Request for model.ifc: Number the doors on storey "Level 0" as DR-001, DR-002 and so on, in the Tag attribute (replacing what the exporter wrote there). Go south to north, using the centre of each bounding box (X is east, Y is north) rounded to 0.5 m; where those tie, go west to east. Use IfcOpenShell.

First a look at what the model holds.

```python
import ifcopenshell
import ifcopenshell.util.element
import ifcopenshell.util.placement

model = ifcopenshell.open("model.ifc")
print(model.schema)
storey = next(s for s in model.by_type("IfcBuildingStorey") if s.Name == "Level 0")
doors = [e for e in ifcopenshell.util.element.get_decomposition(storey) if e.is_a("IfcDoor")]
for e in sorted(doors, key=lambda e: e.id()):
    origin = ifcopenshell.util.placement.get_local_placement(e.ObjectPlacement)[:3, 3]
    print(e.id(), e.Tag, e.Name, origin.round(2) + 0.0, sep=" | ")
```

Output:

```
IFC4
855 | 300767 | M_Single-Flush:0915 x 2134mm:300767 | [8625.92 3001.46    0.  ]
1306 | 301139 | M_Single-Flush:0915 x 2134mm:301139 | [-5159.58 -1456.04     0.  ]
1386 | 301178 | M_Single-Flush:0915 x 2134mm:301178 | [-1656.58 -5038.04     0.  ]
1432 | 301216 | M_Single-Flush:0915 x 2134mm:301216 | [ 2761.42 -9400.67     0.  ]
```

```python
import ifcopenshell
import ifcopenshell.geom
import ifcopenshell.util.element
import ifcopenshell.util.shape

model = ifcopenshell.open("model.ifc")
settings = ifcopenshell.geom.settings()
settings.set("use-world-coords", True)


def centre(element):
    shape = ifcopenshell.geom.create_shape(settings, element)
    return ifcopenshell.util.shape.get_bbox_centroid(shape.geometry)


storey = next(s for s in model.by_type("IfcBuildingStorey") if s.Name == "Level 0")
doors = [e for e in ifcopenshell.util.element.get_decomposition(storey) if e.is_a("IfcDoor")]

# Insertion points can sit at a corner or the storey origin, so sort by the geometry (in metres).
centres = {e: centre(e) for e in doors}
doors.sort(key=lambda e: (round(centres[e][1] / 0.5), centres[e][0]))

for i, e in enumerate(doors, start=1):
    number = f"DR-0{i:02d}"
    e.Tag = number
    print(e.id(), number)

model.write("model_updated.ifc")
```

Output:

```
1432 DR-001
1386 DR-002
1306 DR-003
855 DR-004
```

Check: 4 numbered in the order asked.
